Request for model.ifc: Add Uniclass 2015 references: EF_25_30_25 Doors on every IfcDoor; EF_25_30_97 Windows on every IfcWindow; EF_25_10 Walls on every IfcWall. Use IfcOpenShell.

First a look at what the model holds.

```python
import ifcopenshell

model = ifcopenshell.open("model.ifc")
print(model.schema)
print("classifications:", [c.Name for c in model.by_type("IfcClassification")])
for ifc_class in ("IfcDoor", "IfcRoof", "IfcStair", "IfcWall", "IfcWindow"):
    print(ifc_class, len(model.by_type(ifc_class)))
```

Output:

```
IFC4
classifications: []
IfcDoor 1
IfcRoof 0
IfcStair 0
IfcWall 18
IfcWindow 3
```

```python
import ifcopenshell
import ifcopenshell.api.classification

model = ifcopenshell.open("model.ifc")

system = ifcopenshell.api.classification.add_classification(model, classification="Uniclass 2015")

codes = {
    "IfcDoor": ("EF_25_30_25", "Doors"),
    "IfcWindow": ("EF_25_30_97", "Windows"),
    "IfcWall": ("EF_25_10", "Walls"),
}
for ifc_class, (code, name) in codes.items():
    products = model.by_type(ifc_class)
    ifcopenshell.api.classification.add_reference(
        model, products=products, classification=system, identification=code, name=name
    )
    print(code, len(products))

model.write("model_v2.ifc")
```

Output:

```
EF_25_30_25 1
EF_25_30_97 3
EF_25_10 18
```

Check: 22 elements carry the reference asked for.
